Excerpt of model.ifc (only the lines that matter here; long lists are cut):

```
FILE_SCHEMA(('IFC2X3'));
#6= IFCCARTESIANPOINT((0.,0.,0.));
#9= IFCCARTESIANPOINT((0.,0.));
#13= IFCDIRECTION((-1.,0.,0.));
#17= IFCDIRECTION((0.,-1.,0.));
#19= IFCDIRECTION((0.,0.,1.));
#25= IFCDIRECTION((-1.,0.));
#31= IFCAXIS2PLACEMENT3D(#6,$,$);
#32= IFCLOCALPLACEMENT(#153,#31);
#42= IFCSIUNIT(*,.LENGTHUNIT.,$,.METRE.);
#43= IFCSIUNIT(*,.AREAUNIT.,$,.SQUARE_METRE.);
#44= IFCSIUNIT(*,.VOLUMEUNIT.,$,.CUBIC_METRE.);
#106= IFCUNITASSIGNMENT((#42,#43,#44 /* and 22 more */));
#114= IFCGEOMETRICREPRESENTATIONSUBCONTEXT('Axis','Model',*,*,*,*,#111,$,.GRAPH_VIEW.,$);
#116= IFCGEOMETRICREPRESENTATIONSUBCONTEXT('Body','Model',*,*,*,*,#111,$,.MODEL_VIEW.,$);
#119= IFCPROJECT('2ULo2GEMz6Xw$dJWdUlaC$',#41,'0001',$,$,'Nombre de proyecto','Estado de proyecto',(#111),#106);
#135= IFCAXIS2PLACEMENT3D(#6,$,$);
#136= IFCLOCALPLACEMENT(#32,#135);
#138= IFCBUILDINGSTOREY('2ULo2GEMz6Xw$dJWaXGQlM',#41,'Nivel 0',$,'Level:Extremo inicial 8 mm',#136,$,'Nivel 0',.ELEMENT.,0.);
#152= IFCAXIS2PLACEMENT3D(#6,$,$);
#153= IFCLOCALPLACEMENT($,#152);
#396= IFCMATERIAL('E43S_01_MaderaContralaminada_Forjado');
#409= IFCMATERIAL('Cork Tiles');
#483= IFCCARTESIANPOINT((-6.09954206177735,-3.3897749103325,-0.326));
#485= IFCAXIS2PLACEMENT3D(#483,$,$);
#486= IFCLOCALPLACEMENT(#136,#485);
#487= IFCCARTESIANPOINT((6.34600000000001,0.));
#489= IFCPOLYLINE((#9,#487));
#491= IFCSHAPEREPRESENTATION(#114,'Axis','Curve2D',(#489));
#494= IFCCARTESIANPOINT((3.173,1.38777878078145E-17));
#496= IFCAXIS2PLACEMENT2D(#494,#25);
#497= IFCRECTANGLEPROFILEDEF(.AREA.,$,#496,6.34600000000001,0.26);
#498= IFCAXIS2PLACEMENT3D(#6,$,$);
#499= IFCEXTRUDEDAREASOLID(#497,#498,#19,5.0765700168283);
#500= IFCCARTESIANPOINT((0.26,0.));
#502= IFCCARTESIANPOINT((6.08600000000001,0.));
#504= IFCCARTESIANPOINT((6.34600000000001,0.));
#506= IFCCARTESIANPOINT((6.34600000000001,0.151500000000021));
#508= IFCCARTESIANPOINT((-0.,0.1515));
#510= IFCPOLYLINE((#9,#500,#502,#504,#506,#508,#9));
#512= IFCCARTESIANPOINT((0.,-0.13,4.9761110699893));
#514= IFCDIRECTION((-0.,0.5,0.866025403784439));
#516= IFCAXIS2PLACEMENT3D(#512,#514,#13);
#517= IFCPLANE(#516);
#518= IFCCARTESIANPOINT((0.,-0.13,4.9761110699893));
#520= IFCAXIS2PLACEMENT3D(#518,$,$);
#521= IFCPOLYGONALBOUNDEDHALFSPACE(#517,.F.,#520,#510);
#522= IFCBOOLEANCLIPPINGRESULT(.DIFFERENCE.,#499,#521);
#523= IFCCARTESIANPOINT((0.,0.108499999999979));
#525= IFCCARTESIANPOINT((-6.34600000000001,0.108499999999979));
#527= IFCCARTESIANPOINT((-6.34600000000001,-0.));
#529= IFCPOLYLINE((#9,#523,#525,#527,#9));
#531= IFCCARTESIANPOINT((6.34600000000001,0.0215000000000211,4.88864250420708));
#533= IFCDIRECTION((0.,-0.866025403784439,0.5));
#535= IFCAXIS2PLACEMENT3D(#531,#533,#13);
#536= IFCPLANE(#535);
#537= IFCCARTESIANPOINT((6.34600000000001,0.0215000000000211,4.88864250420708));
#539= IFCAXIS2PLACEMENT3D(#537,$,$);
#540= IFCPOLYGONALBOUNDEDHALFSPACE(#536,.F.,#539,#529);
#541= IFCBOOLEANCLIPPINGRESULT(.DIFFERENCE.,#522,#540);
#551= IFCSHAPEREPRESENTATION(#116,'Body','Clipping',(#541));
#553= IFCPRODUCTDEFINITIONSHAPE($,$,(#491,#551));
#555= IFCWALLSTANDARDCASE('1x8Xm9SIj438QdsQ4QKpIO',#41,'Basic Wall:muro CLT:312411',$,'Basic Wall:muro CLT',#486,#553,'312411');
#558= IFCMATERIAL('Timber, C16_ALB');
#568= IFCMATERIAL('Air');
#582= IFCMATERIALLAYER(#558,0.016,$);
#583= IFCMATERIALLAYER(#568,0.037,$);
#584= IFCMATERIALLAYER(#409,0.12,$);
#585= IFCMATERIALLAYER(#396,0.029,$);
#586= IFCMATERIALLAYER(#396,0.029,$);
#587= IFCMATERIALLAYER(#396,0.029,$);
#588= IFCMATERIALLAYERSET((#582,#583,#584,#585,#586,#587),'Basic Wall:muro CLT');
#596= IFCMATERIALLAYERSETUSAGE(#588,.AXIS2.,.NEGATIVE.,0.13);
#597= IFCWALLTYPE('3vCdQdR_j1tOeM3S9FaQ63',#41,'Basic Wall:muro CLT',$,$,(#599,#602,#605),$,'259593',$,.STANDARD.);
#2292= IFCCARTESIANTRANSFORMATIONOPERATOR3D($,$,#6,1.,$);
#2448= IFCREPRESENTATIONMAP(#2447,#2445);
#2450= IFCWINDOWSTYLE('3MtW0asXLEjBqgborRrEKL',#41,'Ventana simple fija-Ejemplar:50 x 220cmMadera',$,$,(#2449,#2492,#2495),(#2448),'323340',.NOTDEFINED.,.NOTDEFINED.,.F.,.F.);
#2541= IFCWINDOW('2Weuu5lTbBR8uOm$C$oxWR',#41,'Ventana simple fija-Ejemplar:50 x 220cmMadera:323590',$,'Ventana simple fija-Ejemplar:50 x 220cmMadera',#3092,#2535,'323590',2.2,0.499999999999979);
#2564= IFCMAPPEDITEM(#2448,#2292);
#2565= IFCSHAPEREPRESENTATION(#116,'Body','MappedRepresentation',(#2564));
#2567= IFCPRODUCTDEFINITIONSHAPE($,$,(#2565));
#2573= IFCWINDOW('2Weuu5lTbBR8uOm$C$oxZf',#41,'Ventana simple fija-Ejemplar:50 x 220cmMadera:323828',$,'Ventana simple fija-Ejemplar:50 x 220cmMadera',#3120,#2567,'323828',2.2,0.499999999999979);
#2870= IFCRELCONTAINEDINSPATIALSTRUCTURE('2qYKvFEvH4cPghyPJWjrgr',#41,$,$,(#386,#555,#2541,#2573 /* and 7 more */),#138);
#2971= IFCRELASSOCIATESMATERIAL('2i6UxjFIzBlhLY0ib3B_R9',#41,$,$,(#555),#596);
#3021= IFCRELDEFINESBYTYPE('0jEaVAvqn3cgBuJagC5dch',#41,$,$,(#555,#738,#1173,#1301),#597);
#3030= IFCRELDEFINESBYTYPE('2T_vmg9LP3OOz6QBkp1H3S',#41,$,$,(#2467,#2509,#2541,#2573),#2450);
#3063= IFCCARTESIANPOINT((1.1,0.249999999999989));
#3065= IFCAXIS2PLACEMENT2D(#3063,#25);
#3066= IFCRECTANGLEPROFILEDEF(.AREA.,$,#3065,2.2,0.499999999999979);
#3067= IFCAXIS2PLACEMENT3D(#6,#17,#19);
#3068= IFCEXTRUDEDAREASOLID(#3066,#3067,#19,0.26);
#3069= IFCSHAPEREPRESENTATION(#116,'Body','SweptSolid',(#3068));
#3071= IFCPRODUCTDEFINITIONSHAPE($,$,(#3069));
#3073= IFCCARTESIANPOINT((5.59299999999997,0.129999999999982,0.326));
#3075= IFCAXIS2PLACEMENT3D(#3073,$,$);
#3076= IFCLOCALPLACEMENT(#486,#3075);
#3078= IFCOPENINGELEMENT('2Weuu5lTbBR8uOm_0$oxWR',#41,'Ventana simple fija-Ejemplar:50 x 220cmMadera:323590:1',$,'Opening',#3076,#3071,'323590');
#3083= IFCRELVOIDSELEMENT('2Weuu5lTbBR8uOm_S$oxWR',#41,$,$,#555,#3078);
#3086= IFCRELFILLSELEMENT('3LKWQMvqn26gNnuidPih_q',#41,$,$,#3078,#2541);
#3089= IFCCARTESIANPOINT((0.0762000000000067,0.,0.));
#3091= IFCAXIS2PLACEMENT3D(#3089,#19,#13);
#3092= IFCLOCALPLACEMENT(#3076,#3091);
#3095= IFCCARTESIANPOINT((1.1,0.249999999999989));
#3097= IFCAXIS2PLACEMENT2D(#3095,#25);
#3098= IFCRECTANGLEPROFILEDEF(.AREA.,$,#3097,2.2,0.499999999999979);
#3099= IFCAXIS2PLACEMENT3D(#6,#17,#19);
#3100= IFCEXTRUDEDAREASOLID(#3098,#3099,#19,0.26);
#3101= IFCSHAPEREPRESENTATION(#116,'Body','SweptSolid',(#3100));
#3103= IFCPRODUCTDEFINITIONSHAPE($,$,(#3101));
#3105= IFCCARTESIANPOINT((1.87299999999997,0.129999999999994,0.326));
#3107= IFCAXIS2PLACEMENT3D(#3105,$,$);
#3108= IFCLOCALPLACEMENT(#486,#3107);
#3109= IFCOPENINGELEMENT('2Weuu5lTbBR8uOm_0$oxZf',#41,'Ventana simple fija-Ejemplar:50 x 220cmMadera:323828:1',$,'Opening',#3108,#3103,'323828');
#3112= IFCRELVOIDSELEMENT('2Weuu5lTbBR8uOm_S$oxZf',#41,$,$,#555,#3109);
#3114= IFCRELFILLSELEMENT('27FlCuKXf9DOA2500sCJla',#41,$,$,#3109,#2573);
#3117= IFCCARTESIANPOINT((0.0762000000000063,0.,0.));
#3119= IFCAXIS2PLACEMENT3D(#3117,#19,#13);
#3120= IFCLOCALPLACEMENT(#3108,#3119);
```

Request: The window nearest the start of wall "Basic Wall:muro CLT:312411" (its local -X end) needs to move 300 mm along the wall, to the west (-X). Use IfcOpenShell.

```python
import ifcopenshell
import ifcopenshell.api.geometry
import ifcopenshell.util.placement
import ifcopenshell.util.unit

model = ifcopenshell.open("model.ifc")
unit_scale = ifcopenshell.util.unit.calculate_unit_scale(model)

window = model.by_guid("2Weuu5lTbBR8uOm$C$oxZf")
opening = window.FillsVoids[0].RelatingOpeningElement
wall = opening.VoidsElements[0].RelatingBuildingElement

wall_matrix = ifcopenshell.util.placement.get_local_placement(wall.ObjectPlacement)
shift = wall_matrix[:3, 0] * -0.3 / unit_scale
before = ifcopenshell.util.placement.get_local_placement(window.ObjectPlacement)[:3, 3].copy()

# The window is placed relative to its opening, so it follows when the opening moves.
matrix = ifcopenshell.util.placement.get_local_placement(opening.ObjectPlacement)
matrix[:3, 3] += shift
ifcopenshell.api.geometry.edit_object_placement(
    model, product=opening, matrix=matrix, is_si=False, should_transform_children=True
)

after = ifcopenshell.util.placement.get_local_placement(window.ObjectPlacement)[:3, 3]
print("window moved by", (after - before).round(3) + 0.0)

model.write("model_v2.ifc")
```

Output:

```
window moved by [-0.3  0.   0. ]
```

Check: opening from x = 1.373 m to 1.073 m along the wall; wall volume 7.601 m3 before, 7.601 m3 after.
